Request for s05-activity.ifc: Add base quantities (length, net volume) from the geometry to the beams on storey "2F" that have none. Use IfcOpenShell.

First a look at what the model holds.

```python
import ifcopenshell
import ifcopenshell.util.element
import ifcopenshell.util.unit

model = ifcopenshell.open("s05-activity.ifc")
print(model.schema)
for unit_type in ("LENGTHUNIT", "AREAUNIT", "VOLUMEUNIT"):
    print(unit_type, ifcopenshell.util.unit.calculate_unit_scale(model, unit_type))
storey = next(s for s in model.by_type("IfcBuildingStorey") if s.Name == "2F")
beams = [e for e in ifcopenshell.util.element.get_decomposition(storey) if e.is_a("IfcBeam")]
for e in sorted(beams, key=lambda e: e.id()):
    print(e.id(), e.is_a(), e.Name, list(ifcopenshell.util.element.get_psets(e, qtos_only=True)), sep=" | ")
```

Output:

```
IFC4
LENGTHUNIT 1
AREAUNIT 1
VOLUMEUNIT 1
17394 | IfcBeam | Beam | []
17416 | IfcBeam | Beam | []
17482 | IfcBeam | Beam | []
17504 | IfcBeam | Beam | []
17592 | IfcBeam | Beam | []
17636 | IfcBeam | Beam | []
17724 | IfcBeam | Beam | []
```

```python
import ifcopenshell
import ifcopenshell.api.pset
import ifcopenshell.geom
import ifcopenshell.util.element
import ifcopenshell.util.shape
import ifcopenshell.util.unit

model = ifcopenshell.open("s05-activity.ifc")
unit_scale = ifcopenshell.util.unit.calculate_unit_scale(model)
volume_scale = ifcopenshell.util.unit.calculate_unit_scale(model, "VOLUMEUNIT")
settings = ifcopenshell.geom.settings()

storey = next(s for s in model.by_type("IfcBuildingStorey") if s.Name == "2F")
beams = [e for e in ifcopenshell.util.element.get_decomposition(storey) if e.is_a("IfcBeam")]

for e in sorted(beams, key=lambda e: e.id()):
    if ifcopenshell.util.element.get_psets(e, qtos_only=True, should_inherit=False):
        continue
    # Geometry comes back in metres, in the element's own axes.
    shape = ifcopenshell.geom.create_shape(settings, e)
    values = {
        "Length": ifcopenshell.util.shape.get_max_xyz(shape.geometry) / unit_scale,
        "NetVolume": ifcopenshell.util.shape.get_volume(shape.geometry) / volume_scale,
    }
    qto = ifcopenshell.api.pset.add_qto(model, product=e, name="Qto_BeamBaseQuantities")
    ifcopenshell.api.pset.edit_qto(model, qto=qto, properties=values)
    print(e.id(), {k: round(v, 3) for k, v in values.items()})

model.write("s05-activity-out.ifc")
```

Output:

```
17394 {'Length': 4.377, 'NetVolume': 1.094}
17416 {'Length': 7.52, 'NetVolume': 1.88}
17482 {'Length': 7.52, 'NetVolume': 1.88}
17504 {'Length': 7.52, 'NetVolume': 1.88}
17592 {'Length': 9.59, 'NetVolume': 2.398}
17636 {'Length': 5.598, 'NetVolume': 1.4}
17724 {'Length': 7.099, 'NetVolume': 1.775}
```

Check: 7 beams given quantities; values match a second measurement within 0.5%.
